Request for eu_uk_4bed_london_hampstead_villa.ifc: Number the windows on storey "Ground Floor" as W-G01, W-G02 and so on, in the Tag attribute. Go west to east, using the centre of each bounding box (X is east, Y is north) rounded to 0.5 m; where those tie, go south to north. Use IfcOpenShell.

First a look at what the model holds.

```python
import ifcopenshell
import ifcopenshell.util.element
import ifcopenshell.util.placement

model = ifcopenshell.open("eu_uk_4bed_london_hampstead_villa.ifc")
print(model.schema)
storey = next(s for s in model.by_type("IfcBuildingStorey") if s.Name == "Ground Floor")
windows = [e for e in ifcopenshell.util.element.get_decomposition(storey) if e.is_a("IfcWindow")]
for e in sorted(windows, key=lambda e: e.id()):
    origin = ifcopenshell.util.placement.get_local_placement(e.ObjectPlacement)[:3, 3]
    print(e.id(), e.Tag, e.Name, origin.round(2) + 0.0, sep=" | ")
```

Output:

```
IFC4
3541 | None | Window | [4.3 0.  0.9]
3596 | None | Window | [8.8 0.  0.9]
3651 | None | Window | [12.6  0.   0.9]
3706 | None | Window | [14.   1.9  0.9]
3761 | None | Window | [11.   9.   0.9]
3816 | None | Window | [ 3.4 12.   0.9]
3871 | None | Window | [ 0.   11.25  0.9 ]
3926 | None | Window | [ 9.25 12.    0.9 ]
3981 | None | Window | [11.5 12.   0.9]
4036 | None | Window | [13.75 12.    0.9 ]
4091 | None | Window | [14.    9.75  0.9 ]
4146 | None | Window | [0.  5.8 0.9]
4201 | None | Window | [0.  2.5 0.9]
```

```python
import ifcopenshell
import ifcopenshell.geom
import ifcopenshell.util.element
import ifcopenshell.util.shape

model = ifcopenshell.open("eu_uk_4bed_london_hampstead_villa.ifc")
settings = ifcopenshell.geom.settings()
settings.set("use-world-coords", True)


def centre(element):
    shape = ifcopenshell.geom.create_shape(settings, element)
    return ifcopenshell.util.shape.get_bbox_centroid(shape.geometry)


storey = next(s for s in model.by_type("IfcBuildingStorey") if s.Name == "Ground Floor")
windows = [e for e in ifcopenshell.util.element.get_decomposition(storey) if e.is_a("IfcWindow")]

# Insertion points can sit at a corner or the storey origin, so sort by the geometry (in metres).
centres = {e: centre(e) for e in windows}
windows.sort(key=lambda e: (round(centres[e][0] / 0.5), centres[e][1]))

for i, e in enumerate(windows, start=1):
    number = f"W-G{i:02d}"
    e.Tag = number
    print(e.id(), number)

model.write("eu_uk_4bed_london_hampstead_villa_edited.ifc")
```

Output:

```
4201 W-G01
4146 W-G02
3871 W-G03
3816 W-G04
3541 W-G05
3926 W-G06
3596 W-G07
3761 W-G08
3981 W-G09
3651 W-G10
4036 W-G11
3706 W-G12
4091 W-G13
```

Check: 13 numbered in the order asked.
